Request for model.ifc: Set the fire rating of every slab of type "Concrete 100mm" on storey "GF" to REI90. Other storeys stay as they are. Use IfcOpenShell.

First a look at what the model holds.

```python
import ifcopenshell
import ifcopenshell.util.element

model = ifcopenshell.open("model.ifc")
print(model.schema)
storey = next(s for s in model.by_type("IfcBuildingStorey") if s.Name == "GF")
slabs = [e for e in ifcopenshell.util.element.get_decomposition(storey) if e.is_a("IfcSlab")]
seen = {}
for e in slabs:
    element_type = ifcopenshell.util.element.get_type(e)
    key = (element_type.Name if element_type != e and element_type else None, ifcopenshell.util.element.get_pset(e, "Pset_SlabCommon", "FireRating"))
    seen[key] = seen.get(key, 0) + 1
for (name, value), count in sorted(seen.items(), key=str):
    print(count, "x", name, "|", value)
```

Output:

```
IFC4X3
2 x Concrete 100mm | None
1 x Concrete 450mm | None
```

```python
import ifcopenshell
import ifcopenshell.api.pset
import ifcopenshell.util.element

model = ifcopenshell.open("model.ifc")

storey = next(s for s in model.by_type("IfcBuildingStorey") if s.Name == "GF")
slabs = [e for e in ifcopenshell.util.element.get_decomposition(storey) if e.is_a("IfcSlab")]

count = 0
for e in slabs:
    element_type = ifcopenshell.util.element.get_type(e)
    if element_type in (None, e) or element_type.Name != "Concrete 100mm":
        continue
    # add_pset returns the element's existing set when there is one.
    pset = ifcopenshell.api.pset.add_pset(model, product=e, name="Pset_SlabCommon")
    ifcopenshell.api.pset.edit_pset(model, pset=pset, properties={"FireRating": "REI90"})
    count += 1

print(count, "slabs updated")

model.write("model_updated.ifc")
```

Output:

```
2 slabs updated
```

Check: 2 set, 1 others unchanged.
